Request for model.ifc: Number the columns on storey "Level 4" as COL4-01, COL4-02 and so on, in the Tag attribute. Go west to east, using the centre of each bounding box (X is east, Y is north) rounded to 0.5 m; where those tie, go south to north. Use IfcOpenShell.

First a look at what the model holds.

```python
import ifcopenshell
import ifcopenshell.util.element
import ifcopenshell.util.placement

model = ifcopenshell.open("model.ifc")
print(model.schema)
storey = next(s for s in model.by_type("IfcBuildingStorey") if s.Name == "Level 4")
columns = [e for e in ifcopenshell.util.element.get_decomposition(storey) if e.is_a("IfcColumn")]
for e in sorted(columns, key=lambda e: e.id()):
    origin = ifcopenshell.util.placement.get_local_placement(e.ObjectPlacement)[:3, 3]
    print(e.id(), e.Tag, e.Name, origin.round(2) + 0.0, sep=" | ")
```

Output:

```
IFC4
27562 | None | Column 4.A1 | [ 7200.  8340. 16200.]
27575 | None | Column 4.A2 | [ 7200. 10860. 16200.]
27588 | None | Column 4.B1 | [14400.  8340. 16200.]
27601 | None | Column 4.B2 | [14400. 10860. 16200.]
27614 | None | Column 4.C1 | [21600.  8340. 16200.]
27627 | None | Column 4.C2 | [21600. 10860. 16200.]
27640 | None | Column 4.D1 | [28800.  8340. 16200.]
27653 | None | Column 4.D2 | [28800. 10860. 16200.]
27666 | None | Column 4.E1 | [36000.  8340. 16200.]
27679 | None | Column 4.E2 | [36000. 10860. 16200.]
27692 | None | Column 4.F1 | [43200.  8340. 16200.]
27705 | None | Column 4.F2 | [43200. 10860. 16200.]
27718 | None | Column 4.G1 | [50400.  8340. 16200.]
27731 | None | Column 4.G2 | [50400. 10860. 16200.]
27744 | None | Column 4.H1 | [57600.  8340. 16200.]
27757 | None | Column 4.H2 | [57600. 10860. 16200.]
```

```python
import ifcopenshell
import ifcopenshell.geom
import ifcopenshell.util.element
import ifcopenshell.util.shape

model = ifcopenshell.open("model.ifc")
settings = ifcopenshell.geom.settings()
settings.set("use-world-coords", True)


def centre(element):
    shape = ifcopenshell.geom.create_shape(settings, element)
    return ifcopenshell.util.shape.get_bbox_centroid(shape.geometry)


storey = next(s for s in model.by_type("IfcBuildingStorey") if s.Name == "Level 4")
columns = [e for e in ifcopenshell.util.element.get_decomposition(storey) if e.is_a("IfcColumn")]

# Insertion points can sit at a corner or the storey origin, so sort by the geometry (in metres).
centres = {e: centre(e) for e in columns}
columns.sort(key=lambda e: (round(centres[e][0] / 0.5), centres[e][1]))

for i, e in enumerate(columns, start=1):
    number = f"COL4-{i:02d}"
    e.Tag = number
    print(e.id(), number)

model.write("model_updated.ifc")
```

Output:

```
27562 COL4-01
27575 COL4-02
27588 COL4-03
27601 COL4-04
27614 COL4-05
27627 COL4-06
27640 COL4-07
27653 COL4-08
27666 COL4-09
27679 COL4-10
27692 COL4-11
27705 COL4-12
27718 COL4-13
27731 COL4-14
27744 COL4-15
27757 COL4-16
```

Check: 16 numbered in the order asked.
